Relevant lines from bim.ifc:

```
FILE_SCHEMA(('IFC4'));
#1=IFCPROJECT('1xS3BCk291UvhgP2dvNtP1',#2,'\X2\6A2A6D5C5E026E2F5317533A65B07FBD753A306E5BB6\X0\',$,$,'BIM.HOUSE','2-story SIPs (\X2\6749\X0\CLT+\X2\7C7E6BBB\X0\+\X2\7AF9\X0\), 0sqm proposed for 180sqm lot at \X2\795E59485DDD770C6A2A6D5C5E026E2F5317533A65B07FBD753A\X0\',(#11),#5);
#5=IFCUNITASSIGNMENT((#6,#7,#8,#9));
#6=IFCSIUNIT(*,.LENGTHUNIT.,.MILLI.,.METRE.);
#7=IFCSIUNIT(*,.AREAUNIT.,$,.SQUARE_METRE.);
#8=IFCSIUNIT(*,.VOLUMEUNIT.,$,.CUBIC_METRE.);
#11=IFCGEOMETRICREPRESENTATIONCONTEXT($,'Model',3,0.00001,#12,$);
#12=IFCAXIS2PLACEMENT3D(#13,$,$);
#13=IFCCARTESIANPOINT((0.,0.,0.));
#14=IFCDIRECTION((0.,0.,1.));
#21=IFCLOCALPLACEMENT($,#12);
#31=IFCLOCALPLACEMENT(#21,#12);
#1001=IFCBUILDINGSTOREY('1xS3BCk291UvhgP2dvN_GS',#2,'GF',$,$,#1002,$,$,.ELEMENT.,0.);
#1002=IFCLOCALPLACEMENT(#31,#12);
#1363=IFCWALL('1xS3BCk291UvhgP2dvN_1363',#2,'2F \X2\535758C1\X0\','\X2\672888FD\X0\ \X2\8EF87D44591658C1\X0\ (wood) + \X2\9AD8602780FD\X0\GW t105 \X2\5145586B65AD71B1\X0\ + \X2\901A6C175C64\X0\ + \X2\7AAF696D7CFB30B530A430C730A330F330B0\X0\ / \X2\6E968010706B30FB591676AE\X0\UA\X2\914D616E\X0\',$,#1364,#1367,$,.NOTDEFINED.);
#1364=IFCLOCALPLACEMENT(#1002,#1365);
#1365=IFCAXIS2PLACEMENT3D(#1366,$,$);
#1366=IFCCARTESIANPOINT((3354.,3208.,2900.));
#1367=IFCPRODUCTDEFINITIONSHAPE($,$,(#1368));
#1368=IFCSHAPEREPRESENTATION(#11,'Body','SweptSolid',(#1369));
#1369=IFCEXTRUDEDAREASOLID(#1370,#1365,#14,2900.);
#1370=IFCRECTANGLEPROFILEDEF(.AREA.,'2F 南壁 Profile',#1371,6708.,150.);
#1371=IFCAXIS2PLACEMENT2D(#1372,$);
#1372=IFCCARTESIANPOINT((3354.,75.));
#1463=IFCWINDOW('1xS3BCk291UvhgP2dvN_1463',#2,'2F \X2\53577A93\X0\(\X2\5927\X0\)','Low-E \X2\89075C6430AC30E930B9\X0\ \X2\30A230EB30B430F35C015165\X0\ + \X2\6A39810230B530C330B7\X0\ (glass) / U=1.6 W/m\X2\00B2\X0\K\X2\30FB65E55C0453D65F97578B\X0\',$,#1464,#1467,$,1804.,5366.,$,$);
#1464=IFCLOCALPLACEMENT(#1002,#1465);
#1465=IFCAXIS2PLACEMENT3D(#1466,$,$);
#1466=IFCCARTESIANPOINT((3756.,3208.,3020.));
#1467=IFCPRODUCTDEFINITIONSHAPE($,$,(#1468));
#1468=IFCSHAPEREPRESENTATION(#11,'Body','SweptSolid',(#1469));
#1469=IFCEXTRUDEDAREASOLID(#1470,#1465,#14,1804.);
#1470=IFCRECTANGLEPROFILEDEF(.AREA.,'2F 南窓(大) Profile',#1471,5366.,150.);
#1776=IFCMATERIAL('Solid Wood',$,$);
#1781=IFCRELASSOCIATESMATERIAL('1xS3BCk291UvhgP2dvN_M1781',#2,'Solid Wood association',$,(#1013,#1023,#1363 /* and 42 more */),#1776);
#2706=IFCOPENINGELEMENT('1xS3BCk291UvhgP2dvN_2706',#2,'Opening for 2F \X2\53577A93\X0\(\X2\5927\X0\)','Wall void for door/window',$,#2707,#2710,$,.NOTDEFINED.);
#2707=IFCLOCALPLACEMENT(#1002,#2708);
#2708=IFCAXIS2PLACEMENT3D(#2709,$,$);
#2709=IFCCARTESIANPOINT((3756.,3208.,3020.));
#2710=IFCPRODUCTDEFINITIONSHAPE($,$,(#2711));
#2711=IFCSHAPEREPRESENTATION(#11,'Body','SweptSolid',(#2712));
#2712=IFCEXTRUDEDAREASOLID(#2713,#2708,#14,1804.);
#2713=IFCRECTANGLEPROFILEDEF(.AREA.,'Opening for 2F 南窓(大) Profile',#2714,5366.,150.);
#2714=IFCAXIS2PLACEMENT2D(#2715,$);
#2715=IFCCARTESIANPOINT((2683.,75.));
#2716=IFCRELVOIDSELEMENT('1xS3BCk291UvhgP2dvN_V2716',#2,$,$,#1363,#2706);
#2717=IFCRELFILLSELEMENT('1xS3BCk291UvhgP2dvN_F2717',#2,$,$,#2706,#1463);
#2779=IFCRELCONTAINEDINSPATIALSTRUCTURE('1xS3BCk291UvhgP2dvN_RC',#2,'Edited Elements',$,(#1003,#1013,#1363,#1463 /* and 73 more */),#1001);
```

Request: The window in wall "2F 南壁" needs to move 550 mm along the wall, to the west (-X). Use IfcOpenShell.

```python
import ifcopenshell
import ifcopenshell.api.geometry
import ifcopenshell.util.placement
import ifcopenshell.util.unit

model = ifcopenshell.open("bim.ifc")
unit_scale = ifcopenshell.util.unit.calculate_unit_scale(model)

window = model.by_id(1463)
opening = window.FillsVoids[0].RelatingOpeningElement
wall = opening.VoidsElements[0].RelatingBuildingElement

wall_matrix = ifcopenshell.util.placement.get_local_placement(wall.ObjectPlacement)
shift = wall_matrix[:3, 0] * -0.55 / unit_scale
before = ifcopenshell.util.placement.get_local_placement(window.ObjectPlacement)[:3, 3].copy()

# The window is not placed relative to its opening, so move both.
for product in (opening, window):
    matrix = ifcopenshell.util.placement.get_local_placement(product.ObjectPlacement)
    matrix[:3, 3] += shift
    ifcopenshell.api.geometry.edit_object_placement(model, product=product, matrix=matrix, is_si=False)

after = ifcopenshell.util.placement.get_local_placement(window.ObjectPlacement)[:3, 3]
print("window moved by", (after - before).round(3) + 0.0)

model.write("bim_rev.ifc")
```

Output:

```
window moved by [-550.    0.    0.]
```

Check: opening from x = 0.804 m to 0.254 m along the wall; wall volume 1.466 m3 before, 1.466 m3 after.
